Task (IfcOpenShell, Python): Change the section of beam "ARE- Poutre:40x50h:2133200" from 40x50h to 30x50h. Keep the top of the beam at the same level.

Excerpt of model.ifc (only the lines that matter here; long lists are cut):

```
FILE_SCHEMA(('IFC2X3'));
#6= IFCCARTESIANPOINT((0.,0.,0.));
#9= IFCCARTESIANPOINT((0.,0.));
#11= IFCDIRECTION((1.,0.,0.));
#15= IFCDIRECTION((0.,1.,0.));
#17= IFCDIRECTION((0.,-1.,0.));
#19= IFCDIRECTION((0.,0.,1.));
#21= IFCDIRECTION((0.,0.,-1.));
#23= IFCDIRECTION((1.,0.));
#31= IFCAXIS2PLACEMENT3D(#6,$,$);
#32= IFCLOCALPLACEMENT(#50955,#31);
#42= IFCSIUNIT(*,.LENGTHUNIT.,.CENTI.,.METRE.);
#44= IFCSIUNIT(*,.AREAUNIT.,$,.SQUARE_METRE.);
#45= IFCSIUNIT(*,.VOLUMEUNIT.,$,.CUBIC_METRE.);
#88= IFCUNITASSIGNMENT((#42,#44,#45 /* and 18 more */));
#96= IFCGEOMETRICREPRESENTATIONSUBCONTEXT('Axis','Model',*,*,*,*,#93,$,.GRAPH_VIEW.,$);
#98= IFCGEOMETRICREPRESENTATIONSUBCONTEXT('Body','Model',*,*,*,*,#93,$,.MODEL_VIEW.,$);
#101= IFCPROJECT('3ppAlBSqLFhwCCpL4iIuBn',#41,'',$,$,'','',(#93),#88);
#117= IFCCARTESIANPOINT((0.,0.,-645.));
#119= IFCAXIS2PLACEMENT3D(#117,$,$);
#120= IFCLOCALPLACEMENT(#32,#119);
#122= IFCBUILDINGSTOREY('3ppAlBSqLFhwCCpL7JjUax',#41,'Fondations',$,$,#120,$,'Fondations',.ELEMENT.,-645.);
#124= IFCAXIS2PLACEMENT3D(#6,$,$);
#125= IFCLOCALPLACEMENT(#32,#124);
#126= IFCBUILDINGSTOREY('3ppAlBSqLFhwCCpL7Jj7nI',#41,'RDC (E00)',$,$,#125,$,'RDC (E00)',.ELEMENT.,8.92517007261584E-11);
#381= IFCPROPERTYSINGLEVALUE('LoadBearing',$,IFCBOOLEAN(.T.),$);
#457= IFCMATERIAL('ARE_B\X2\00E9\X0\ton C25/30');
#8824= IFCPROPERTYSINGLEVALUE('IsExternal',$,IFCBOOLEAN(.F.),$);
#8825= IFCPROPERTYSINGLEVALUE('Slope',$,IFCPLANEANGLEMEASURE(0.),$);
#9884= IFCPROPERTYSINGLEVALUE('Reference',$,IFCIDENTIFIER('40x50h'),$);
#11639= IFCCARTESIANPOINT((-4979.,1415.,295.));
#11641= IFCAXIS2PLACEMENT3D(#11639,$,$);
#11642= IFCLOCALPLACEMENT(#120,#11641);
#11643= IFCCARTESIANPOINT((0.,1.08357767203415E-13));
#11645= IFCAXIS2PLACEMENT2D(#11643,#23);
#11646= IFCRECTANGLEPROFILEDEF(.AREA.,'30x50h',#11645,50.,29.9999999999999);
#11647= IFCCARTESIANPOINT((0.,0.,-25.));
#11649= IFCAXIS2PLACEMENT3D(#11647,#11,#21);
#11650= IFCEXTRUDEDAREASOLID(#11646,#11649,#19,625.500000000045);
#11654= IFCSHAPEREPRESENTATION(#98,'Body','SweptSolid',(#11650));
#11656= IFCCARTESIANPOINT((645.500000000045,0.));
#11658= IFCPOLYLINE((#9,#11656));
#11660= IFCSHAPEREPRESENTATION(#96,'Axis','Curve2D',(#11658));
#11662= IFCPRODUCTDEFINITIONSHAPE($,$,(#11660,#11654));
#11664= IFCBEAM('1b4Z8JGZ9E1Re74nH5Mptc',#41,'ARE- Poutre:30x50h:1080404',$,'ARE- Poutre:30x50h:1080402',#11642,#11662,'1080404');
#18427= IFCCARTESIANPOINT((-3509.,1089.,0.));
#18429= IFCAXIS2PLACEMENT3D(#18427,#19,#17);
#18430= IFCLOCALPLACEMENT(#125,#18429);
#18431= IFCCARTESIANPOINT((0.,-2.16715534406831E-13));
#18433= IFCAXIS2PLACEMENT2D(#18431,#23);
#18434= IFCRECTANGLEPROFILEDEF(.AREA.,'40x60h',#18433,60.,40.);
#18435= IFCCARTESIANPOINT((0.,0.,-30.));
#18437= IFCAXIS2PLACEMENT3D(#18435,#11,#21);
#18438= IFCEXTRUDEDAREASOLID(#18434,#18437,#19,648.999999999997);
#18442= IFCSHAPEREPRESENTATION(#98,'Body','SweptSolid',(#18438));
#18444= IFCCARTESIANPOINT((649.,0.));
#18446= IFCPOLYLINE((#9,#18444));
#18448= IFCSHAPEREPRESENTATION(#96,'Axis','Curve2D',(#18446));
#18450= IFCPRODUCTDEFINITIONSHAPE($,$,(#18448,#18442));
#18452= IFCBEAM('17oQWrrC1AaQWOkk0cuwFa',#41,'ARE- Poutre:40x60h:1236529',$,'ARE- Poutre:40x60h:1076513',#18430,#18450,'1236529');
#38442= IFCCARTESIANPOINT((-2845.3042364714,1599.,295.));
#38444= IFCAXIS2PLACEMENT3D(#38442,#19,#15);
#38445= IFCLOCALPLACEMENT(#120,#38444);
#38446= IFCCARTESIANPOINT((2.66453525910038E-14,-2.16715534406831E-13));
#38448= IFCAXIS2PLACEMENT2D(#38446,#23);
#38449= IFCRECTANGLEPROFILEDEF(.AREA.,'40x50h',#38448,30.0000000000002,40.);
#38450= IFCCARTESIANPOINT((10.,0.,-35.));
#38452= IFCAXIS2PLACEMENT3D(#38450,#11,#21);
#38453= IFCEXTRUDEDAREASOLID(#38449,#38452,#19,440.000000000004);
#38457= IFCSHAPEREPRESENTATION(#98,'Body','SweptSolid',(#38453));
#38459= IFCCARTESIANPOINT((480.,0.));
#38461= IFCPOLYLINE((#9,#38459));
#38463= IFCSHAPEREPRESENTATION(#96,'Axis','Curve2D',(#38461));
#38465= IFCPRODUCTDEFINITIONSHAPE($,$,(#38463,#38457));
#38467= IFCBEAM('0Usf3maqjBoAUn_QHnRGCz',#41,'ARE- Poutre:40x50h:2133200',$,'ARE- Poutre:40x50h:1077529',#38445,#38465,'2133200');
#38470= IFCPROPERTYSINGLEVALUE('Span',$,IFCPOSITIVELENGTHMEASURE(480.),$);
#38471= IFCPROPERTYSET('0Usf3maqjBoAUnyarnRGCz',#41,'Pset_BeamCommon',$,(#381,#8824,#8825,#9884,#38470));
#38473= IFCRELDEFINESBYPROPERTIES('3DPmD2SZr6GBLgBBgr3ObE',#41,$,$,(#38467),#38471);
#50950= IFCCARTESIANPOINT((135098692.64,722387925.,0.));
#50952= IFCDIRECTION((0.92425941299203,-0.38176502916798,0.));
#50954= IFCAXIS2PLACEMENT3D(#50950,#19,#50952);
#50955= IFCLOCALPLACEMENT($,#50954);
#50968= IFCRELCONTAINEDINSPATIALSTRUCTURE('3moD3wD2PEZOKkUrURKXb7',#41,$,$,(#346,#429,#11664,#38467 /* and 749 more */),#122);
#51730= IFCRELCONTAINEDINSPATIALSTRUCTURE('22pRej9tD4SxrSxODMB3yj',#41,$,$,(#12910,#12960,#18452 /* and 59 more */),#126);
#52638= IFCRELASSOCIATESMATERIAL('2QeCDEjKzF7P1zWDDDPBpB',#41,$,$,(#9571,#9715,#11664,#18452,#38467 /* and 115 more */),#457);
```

```python
import ifcopenshell
import ifcopenshell.api.pset
import ifcopenshell.util.element
import ifcopenshell.util.representation

model = ifcopenshell.open("model.ifc")

member = model.by_guid("0Usf3maqjBoAUn_QHnRGCz")
source = next(p for p in model.by_type("IfcRectangleProfileDef") if p.ProfileName == "30x50h")

body = ifcopenshell.util.representation.get_representation(member, "Model", "Body")
solid = body.Items[0]
old_profile = solid.SweptArea

# Copy the section's sizes but keep this member's own profile position.
profile = ifcopenshell.util.element.copy(model, source)
# Profiles are centred, so shift by half the change in depth to hold the top.
shift = (old_profile.XDim - profile.XDim) / 2
x, y = old_profile.Position.Location.Coordinates
up = (-1.0, 0.0)  # upwards, in the solid's own plane
location = model.createIfcCartesianPoint((x + up[0] * shift, y + up[1] * shift))
profile.Position = model.createIfcAxis2Placement2D(location, old_profile.Position.RefDirection)
solid.SweptArea = profile
if not model.get_total_inverses(old_profile):
    ifcopenshell.util.element.remove_deep2(model, old_profile)
member.Name = member.Name.replace("40x50h", "30x50h")
member.ObjectType = member.ObjectType.replace("40x50h", "30x50h")
pset = model.by_id(ifcopenshell.util.element.get_pset(member, "Pset_BeamCommon", should_inherit=False)["id"])
ifcopenshell.api.pset.edit_pset(model, pset=pset, properties={"Reference": "30x50h"})

print(solid.SweptArea)

model.write("model_edited.ifc")
```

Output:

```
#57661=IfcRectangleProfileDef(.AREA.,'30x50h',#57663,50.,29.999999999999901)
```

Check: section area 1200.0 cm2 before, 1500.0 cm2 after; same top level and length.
